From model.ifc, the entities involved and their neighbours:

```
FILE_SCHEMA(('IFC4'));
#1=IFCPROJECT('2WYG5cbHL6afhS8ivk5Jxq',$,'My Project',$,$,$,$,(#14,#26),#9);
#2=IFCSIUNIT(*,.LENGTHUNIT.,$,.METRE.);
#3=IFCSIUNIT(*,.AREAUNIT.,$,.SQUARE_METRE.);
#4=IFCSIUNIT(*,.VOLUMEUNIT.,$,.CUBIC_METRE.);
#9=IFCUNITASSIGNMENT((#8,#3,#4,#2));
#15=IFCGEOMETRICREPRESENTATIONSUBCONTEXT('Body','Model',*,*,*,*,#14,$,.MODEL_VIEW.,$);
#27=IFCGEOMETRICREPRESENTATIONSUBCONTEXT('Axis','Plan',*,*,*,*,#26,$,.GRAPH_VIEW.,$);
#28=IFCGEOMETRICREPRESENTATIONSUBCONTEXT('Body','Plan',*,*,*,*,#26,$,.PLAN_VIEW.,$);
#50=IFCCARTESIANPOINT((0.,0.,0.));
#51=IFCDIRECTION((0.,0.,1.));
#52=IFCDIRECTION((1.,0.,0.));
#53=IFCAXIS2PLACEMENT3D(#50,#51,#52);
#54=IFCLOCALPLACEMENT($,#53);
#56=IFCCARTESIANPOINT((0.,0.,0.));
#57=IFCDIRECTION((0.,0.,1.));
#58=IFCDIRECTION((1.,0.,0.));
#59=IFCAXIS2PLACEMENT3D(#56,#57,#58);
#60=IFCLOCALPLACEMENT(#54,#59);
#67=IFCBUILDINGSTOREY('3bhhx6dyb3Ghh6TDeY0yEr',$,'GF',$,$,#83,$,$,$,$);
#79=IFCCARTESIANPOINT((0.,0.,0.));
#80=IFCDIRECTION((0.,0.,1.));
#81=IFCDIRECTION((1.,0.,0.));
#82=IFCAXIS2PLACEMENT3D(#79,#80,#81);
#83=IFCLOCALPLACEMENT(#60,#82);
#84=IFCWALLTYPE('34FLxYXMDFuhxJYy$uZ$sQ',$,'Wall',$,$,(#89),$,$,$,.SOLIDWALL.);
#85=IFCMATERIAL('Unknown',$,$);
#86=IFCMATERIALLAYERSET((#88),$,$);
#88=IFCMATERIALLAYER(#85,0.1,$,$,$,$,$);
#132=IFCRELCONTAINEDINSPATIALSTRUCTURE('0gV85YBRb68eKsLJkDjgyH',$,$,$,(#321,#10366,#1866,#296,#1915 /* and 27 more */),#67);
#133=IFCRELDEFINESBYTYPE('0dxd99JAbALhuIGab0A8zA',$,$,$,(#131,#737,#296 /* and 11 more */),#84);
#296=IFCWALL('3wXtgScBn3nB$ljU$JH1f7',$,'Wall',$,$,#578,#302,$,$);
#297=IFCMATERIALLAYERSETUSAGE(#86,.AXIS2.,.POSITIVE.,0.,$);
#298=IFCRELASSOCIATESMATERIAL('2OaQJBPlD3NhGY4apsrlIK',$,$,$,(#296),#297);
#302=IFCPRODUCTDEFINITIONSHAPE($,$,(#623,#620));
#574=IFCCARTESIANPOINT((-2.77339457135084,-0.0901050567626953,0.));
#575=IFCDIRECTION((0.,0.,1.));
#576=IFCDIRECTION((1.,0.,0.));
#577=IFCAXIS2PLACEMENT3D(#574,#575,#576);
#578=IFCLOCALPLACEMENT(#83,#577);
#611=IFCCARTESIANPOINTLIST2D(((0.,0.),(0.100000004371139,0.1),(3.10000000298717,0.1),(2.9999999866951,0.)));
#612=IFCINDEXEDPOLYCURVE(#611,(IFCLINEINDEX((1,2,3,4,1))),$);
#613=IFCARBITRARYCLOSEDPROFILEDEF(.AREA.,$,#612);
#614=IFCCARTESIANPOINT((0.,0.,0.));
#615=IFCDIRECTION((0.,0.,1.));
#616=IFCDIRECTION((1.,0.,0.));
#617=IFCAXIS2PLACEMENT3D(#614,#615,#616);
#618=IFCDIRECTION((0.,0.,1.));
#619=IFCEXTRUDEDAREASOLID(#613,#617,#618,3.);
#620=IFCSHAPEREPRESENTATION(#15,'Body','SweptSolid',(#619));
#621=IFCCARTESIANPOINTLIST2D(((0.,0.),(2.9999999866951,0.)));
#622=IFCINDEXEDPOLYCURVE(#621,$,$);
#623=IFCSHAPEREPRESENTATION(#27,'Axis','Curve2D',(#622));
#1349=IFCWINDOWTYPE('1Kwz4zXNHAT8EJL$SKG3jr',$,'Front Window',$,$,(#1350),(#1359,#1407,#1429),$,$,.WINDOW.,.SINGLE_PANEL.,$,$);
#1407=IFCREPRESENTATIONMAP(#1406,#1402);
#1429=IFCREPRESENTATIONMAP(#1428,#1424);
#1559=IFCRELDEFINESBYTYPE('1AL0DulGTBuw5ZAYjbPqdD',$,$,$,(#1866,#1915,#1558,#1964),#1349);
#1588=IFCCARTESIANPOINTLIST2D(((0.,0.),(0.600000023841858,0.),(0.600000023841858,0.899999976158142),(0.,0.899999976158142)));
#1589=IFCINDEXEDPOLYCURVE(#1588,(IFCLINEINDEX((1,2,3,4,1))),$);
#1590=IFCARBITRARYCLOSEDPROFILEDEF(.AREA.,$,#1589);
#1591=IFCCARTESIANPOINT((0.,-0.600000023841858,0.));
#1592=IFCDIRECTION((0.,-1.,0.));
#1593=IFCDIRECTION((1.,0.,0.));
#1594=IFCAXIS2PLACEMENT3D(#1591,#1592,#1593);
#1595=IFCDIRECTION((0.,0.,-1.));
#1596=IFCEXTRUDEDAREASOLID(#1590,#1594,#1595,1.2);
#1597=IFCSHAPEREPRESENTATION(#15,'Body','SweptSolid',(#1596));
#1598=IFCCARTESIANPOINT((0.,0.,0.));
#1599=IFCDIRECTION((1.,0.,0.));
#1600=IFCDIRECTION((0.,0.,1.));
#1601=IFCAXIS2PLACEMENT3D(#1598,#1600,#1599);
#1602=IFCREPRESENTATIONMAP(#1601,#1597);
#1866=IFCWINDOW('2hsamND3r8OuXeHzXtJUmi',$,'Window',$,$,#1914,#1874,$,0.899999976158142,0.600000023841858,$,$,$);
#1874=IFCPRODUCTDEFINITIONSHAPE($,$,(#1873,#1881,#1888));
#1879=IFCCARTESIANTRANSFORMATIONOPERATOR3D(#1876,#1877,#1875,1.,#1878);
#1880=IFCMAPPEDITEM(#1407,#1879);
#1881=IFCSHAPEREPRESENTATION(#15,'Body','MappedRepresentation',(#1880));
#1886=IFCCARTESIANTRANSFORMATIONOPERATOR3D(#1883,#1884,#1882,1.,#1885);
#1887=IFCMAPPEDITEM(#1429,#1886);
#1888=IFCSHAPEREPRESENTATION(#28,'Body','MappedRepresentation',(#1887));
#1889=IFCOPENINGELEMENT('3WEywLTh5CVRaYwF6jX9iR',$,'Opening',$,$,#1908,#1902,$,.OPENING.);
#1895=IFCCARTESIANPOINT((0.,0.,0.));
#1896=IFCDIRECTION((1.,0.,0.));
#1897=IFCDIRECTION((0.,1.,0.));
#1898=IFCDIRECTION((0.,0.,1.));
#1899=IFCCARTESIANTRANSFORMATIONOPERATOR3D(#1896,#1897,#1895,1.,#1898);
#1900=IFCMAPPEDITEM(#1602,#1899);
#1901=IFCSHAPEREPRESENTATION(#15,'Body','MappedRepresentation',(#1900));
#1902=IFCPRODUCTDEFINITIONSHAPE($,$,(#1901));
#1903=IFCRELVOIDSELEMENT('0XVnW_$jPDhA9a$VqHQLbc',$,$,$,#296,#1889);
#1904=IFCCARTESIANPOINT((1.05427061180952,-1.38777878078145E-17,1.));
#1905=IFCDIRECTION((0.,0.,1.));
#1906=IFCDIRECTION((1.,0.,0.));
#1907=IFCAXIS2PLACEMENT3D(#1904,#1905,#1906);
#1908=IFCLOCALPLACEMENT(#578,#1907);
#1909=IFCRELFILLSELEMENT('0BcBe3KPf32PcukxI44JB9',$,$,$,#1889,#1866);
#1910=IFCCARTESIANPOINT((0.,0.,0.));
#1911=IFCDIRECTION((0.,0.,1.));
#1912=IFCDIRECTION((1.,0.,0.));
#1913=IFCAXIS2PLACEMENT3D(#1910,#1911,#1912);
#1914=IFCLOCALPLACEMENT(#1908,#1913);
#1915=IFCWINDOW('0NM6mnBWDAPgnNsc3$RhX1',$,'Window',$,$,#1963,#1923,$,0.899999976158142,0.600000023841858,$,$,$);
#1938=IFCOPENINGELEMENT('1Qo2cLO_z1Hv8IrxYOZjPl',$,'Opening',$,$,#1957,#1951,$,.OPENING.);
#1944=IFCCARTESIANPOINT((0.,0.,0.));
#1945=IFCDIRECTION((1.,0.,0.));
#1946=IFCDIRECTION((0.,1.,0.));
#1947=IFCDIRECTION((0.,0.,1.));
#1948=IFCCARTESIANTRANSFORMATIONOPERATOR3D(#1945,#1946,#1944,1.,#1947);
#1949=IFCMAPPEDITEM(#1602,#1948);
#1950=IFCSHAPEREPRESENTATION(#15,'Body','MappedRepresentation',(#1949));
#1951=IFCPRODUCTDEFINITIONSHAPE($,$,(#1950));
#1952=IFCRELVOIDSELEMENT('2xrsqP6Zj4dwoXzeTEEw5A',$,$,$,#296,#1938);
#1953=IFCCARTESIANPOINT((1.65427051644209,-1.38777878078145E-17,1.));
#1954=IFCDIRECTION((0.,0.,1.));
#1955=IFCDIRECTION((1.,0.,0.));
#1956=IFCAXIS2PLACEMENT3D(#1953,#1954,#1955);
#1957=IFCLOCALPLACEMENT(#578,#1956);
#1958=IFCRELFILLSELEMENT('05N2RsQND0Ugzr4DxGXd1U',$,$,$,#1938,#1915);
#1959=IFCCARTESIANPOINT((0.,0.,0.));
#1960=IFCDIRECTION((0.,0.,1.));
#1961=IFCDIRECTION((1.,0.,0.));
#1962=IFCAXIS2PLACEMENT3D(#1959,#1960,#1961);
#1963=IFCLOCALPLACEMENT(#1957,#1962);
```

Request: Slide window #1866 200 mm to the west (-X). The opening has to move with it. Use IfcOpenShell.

```python
import ifcopenshell
import ifcopenshell.api.geometry
import ifcopenshell.util.placement
import ifcopenshell.util.unit

model = ifcopenshell.open("model.ifc")
unit_scale = ifcopenshell.util.unit.calculate_unit_scale(model)

window = model.by_id(1866)
opening = window.FillsVoids[0].RelatingOpeningElement
wall = opening.VoidsElements[0].RelatingBuildingElement

wall_matrix = ifcopenshell.util.placement.get_local_placement(wall.ObjectPlacement)
shift = wall_matrix[:3, 0] * -0.2 / unit_scale
before = ifcopenshell.util.placement.get_local_placement(window.ObjectPlacement)[:3, 3].copy()

# The window is placed relative to its opening, so it follows when the opening moves.
matrix = ifcopenshell.util.placement.get_local_placement(opening.ObjectPlacement)
matrix[:3, 3] += shift
ifcopenshell.api.geometry.edit_object_placement(
    model, product=opening, matrix=matrix, is_si=False, should_transform_children=True
)

after = ifcopenshell.util.placement.get_local_placement(window.ObjectPlacement)[:3, 3]
print("window moved by", (after - before).round(3) + 0.0)

model.write("model_updated.ifc")
```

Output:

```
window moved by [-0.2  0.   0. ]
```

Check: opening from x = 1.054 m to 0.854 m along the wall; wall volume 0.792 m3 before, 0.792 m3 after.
